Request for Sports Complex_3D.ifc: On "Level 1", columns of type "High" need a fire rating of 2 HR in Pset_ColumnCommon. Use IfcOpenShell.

First a look at what the model holds.

```python
import ifcopenshell
import ifcopenshell.util.element

model = ifcopenshell.open("Sports Complex_3D.ifc")
print(model.schema)
storey = next(s for s in model.by_type("IfcBuildingStorey") if s.Name == "Level 1")
columns = [e for e in ifcopenshell.util.element.get_decomposition(storey) if e.is_a("IfcColumn")]
seen = {}
for e in columns:
    element_type = ifcopenshell.util.element.get_type(e)
    key = (element_type.Name if element_type != e and element_type else None, ifcopenshell.util.element.get_pset(e, "Pset_ColumnCommon", "FireRating"))
    seen[key] = seen.get(key, 0) + 1
for (name, value), count in sorted(seen.items(), key=str):
    print(count, "x", name, "|", value)
```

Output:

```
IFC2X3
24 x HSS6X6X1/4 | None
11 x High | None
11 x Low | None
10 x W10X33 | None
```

```python
import ifcopenshell
import ifcopenshell.api.pset
import ifcopenshell.util.element

model = ifcopenshell.open("Sports Complex_3D.ifc")

storey = next(s for s in model.by_type("IfcBuildingStorey") if s.Name == "Level 1")
columns = [e for e in ifcopenshell.util.element.get_decomposition(storey) if e.is_a("IfcColumn")]

count = 0
for e in columns:
    element_type = ifcopenshell.util.element.get_type(e)
    if element_type in (None, e) or element_type.Name != "High":
        continue
    # add_pset returns the element's existing set when there is one.
    pset = ifcopenshell.api.pset.add_pset(model, product=e, name="Pset_ColumnCommon")
    ifcopenshell.api.pset.edit_pset(model, pset=pset, properties={"FireRating": "2 HR"})
    count += 1

print(count, "columns updated")

model.write("Sports Complex_3D_edited.ifc")
```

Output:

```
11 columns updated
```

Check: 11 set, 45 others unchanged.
